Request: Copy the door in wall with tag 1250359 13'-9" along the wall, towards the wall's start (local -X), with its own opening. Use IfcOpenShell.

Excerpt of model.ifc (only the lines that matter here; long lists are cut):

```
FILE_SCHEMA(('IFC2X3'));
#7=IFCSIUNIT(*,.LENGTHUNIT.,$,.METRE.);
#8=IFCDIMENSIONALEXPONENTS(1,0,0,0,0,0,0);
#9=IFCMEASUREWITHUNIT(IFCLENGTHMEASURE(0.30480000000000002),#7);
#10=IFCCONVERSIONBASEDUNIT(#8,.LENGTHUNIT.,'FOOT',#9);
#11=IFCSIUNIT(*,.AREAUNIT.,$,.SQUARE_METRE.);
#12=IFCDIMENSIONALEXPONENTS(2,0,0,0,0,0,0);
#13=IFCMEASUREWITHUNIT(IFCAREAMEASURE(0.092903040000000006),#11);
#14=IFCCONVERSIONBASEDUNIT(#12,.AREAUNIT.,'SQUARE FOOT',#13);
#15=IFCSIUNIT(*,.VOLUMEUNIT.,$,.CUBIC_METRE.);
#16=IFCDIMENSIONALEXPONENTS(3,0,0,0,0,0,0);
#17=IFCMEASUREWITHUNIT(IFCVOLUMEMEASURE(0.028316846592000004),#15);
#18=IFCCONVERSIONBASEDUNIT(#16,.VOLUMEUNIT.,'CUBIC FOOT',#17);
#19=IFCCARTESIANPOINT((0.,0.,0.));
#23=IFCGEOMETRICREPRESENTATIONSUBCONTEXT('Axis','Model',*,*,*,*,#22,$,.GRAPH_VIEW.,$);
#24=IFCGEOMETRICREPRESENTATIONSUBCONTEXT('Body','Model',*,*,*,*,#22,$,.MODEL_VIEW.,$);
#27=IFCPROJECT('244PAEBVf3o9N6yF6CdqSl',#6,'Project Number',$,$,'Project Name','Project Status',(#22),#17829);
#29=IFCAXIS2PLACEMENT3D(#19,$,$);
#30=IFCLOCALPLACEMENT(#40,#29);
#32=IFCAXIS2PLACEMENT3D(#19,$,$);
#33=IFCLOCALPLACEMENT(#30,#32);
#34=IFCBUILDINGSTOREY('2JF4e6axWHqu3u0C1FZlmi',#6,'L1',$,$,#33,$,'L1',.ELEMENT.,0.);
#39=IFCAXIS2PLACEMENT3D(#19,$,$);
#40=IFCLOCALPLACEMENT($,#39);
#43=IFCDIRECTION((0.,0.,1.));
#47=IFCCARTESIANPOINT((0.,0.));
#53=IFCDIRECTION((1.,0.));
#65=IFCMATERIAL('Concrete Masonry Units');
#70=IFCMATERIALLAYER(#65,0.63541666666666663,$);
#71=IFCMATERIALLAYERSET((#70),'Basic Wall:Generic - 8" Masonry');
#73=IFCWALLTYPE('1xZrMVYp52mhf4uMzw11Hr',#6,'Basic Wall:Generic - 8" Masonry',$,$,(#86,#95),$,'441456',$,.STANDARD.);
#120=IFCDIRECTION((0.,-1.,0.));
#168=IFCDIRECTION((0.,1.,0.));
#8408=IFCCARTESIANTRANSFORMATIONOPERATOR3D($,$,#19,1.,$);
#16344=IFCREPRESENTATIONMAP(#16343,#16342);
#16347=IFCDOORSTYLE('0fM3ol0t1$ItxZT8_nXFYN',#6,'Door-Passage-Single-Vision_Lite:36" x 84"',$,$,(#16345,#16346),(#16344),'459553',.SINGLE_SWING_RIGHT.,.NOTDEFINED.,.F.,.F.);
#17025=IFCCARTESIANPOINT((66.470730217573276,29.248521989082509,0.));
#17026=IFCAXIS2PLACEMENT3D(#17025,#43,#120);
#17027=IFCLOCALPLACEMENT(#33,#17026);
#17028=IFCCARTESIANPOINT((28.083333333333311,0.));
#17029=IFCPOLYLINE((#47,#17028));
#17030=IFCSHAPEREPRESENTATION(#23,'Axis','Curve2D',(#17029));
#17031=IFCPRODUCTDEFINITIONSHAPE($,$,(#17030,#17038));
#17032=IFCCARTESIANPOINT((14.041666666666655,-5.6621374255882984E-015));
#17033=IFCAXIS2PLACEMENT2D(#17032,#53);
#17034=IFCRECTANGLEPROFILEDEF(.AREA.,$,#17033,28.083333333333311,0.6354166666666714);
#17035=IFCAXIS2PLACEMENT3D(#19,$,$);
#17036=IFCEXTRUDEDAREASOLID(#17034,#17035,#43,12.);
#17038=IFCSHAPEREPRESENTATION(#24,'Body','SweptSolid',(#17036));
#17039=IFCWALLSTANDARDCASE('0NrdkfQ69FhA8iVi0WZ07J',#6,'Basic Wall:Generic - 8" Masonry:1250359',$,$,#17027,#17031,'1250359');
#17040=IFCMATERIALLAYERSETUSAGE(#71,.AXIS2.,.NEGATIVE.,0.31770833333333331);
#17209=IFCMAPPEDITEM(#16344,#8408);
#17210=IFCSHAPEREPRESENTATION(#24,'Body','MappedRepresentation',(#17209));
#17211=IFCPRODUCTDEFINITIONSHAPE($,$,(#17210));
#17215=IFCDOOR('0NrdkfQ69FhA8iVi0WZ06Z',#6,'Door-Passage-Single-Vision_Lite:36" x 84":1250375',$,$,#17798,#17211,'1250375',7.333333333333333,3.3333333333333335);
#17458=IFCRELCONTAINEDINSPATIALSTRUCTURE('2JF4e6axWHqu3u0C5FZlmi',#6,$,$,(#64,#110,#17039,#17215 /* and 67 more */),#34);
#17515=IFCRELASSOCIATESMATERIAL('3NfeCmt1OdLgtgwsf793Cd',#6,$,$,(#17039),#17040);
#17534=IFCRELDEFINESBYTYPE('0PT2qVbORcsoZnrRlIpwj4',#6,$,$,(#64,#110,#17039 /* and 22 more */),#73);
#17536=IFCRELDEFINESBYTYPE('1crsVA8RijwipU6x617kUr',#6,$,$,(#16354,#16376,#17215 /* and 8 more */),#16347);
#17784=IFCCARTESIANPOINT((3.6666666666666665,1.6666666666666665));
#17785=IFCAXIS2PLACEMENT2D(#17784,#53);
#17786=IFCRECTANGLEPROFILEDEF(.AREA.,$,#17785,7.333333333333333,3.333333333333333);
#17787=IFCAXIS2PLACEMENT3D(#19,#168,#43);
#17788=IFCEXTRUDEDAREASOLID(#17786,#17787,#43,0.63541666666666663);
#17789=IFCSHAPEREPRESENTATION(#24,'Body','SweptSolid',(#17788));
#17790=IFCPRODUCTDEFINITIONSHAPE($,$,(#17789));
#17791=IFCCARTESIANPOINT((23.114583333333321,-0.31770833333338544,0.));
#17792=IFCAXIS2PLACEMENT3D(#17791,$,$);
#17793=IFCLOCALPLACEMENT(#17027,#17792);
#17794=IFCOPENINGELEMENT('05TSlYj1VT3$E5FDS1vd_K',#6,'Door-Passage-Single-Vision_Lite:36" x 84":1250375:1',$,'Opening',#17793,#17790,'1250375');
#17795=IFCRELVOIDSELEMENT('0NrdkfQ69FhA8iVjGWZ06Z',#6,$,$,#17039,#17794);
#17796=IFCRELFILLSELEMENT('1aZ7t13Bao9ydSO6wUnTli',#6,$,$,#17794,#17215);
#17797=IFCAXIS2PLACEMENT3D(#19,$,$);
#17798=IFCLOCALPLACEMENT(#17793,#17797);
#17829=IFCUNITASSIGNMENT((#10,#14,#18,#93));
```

```python
import ifcopenshell
import ifcopenshell.api.feature
import ifcopenshell.api.geometry
import ifcopenshell.api.root
import ifcopenshell.geom
import ifcopenshell.util.element
import ifcopenshell.util.placement
import ifcopenshell.util.shape
import ifcopenshell.util.unit

model = ifcopenshell.open("model.ifc")
unit_scale = ifcopenshell.util.unit.calculate_unit_scale(model)
settings = ifcopenshell.geom.settings()


def volume(element):
    """Net volume in cubic metres, openings subtracted."""
    shape = ifcopenshell.geom.create_shape(settings, element)
    return ifcopenshell.util.shape.get_volume(shape.geometry)


def reuse_history(source, copy):
    """copy_class also copies each property set's owner history, people and application; keep the originals."""
    for rel in copy.IsDefinedBy:
        if rel.is_a("IfcRelDefinesByProperties") and (history := rel.RelatingPropertyDefinition.OwnerHistory):
            rel.RelatingPropertyDefinition.OwnerHistory = source.OwnerHistory
            ifcopenshell.util.element.remove_deep2(model, history)


door = model.by_id(17215)
opening = door.FillsVoids[0].RelatingOpeningElement
wall = opening.VoidsElements[0].RelatingBuildingElement
before = volume(wall)
shift = ifcopenshell.util.placement.get_local_placement(wall.ObjectPlacement)[:3, 0] * -165 * 0.0254 / unit_scale

# copy_class copies the void relationship, type, container and properties, but no geometry.
new_opening = ifcopenshell.api.root.copy_class(model, product=opening)
new_opening.Representation = ifcopenshell.util.element.copy_deep(
    model, opening.Representation, exclude=["IfcGeometricRepresentationContext", "IfcRepresentationMap"]
)
new_opening.Name = 'Door-Passage-Single-Vision_Lite:36" x 84"'
new_opening.Tag = None
new_door = ifcopenshell.api.root.copy_class(model, product=door)
new_door.Representation = ifcopenshell.util.element.copy_deep(
    model, door.Representation, exclude=["IfcGeometricRepresentationContext", "IfcRepresentationMap"]
)
new_door.Name = 'Door-Passage-Single-Vision_Lite:36" x 84"'
new_door.Tag = None
reuse_history(door, new_door)
fills = ifcopenshell.api.feature.add_filling(model, opening=new_opening, element=new_door)
fills.OwnerHistory = new_door.OwnerHistory  # required in IFC2X3

for old, new in ((opening, new_opening), (door, new_door)):
    matrix = ifcopenshell.util.placement.get_local_placement(old.ObjectPlacement)
    matrix[:3, 3] += shift
    ifcopenshell.api.geometry.edit_object_placement(model, product=new, matrix=matrix, is_si=False)

after = volume(wall)

print(f"wall volume {before:.3f} -> {after:.3f} m3")

model.write("model_v2.ifc")
```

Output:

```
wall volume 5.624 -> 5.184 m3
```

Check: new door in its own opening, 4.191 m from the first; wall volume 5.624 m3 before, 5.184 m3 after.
